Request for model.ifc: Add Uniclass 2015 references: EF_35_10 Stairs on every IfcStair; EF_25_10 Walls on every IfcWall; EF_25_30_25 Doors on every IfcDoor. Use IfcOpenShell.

First a look at what the model holds.

```python
import ifcopenshell

model = ifcopenshell.open("model.ifc")
print(model.schema)
print("classifications:", [c.Name for c in model.by_type("IfcClassification")])
for ifc_class in ("IfcDoor", "IfcRoof", "IfcStair", "IfcWall", "IfcWindow"):
    print(ifc_class, len(model.by_type(ifc_class)))
```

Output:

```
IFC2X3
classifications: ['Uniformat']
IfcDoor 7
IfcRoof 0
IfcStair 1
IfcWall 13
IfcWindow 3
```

```python
import ifcopenshell
import ifcopenshell.api.classification

model = ifcopenshell.open("model.ifc")

# IFC2X3 requires Source and Edition and has no link from the project to the system.
system = model.create_entity("IfcClassification", Source="NBS", Edition="2015", Name="Uniclass 2015")

codes = {
    "IfcStair": ("EF_35_10", "Stairs"),
    "IfcWall": ("EF_25_10", "Walls"),
    "IfcDoor": ("EF_25_30_25", "Doors"),
}
for ifc_class, (code, name) in codes.items():
    products = model.by_type(ifc_class)
    ifcopenshell.api.classification.add_reference(
        model, products=products, classification=system, identification=code, name=name
    )
    print(code, len(products))

model.write("model_rev.ifc")
```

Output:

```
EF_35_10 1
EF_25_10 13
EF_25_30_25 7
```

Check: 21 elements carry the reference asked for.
